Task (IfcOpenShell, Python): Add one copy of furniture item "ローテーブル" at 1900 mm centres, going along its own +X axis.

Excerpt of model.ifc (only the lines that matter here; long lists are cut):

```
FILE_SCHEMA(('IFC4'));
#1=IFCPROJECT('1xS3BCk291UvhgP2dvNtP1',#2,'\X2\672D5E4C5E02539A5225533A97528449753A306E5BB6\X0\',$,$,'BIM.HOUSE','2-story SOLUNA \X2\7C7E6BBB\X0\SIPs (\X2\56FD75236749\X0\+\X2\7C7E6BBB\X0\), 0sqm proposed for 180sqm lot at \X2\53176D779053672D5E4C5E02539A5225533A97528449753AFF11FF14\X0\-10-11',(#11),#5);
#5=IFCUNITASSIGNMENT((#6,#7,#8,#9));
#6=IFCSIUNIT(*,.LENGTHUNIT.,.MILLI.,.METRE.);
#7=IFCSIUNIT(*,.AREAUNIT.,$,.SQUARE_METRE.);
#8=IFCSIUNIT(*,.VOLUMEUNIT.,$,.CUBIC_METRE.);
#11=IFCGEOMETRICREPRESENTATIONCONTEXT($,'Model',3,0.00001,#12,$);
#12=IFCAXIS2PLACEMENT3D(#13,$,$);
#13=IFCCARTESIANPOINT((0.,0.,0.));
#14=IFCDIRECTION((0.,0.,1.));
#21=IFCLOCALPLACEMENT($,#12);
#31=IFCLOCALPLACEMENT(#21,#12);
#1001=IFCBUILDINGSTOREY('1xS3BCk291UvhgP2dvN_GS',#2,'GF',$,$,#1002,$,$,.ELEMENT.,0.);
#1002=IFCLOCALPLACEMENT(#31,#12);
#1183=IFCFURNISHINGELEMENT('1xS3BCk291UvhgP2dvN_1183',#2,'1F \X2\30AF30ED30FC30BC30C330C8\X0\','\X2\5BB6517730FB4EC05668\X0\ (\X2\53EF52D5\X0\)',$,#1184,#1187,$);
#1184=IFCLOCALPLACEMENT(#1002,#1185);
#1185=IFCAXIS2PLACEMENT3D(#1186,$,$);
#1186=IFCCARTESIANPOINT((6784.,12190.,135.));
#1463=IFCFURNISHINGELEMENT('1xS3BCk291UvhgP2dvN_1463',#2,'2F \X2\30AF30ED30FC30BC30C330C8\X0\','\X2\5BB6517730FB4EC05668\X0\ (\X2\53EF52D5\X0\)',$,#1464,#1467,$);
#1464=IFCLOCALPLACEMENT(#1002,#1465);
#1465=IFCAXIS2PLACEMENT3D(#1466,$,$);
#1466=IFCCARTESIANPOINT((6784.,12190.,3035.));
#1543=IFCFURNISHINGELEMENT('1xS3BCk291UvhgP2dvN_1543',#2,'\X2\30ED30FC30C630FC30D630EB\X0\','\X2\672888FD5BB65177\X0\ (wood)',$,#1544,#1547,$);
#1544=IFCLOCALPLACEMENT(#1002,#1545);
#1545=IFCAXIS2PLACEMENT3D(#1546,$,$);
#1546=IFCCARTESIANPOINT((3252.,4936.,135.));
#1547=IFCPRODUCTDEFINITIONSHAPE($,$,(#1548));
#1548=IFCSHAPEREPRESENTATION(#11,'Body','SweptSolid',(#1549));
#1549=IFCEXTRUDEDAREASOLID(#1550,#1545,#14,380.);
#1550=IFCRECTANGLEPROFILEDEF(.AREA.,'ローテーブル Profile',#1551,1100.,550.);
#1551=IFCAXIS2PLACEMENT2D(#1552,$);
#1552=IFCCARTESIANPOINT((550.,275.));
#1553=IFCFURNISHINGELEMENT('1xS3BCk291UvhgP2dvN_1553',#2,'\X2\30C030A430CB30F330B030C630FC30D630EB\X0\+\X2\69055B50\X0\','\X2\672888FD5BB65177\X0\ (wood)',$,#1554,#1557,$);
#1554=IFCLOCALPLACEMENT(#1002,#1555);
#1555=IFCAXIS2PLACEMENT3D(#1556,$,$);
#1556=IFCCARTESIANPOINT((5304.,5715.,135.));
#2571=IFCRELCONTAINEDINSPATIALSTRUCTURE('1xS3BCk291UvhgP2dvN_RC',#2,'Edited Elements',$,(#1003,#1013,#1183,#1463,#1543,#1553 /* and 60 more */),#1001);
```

```python
import ifcopenshell
import ifcopenshell.api.geometry
import ifcopenshell.api.root
import ifcopenshell.util.element
import ifcopenshell.util.placement
import ifcopenshell.util.unit

model = ifcopenshell.open("model.ifc")
unit_scale = ifcopenshell.util.unit.calculate_unit_scale(model)


def reuse_history(source, copy):
    """copy_class also copies each property set's owner history, people and application; keep the originals."""
    for rel in copy.IsDefinedBy:
        if rel.is_a("IfcRelDefinesByProperties") and (history := rel.RelatingPropertyDefinition.OwnerHistory):
            rel.RelatingPropertyDefinition.OwnerHistory = source.OwnerHistory
            ifcopenshell.util.element.remove_deep2(model, history)


source = model.by_id(1543)
base = ifcopenshell.util.placement.get_local_placement(source.ObjectPlacement)
step = base[:3, 0] * 1.9 / unit_scale

for i in range(1, 2):
    copy = ifcopenshell.api.root.copy_class(model, product=source)
    copy.Representation = ifcopenshell.util.element.copy_deep(
        model, source.Representation, exclude=["IfcGeometricRepresentationContext", "IfcRepresentationMap"]
    )
    reuse_history(source, copy)
    matrix = base.copy()
    matrix[:3, 3] += i * step
    print("added at", matrix[:3, 3].round(3) + 0.0)
    ifcopenshell.api.geometry.edit_object_placement(model, product=copy, matrix=matrix, is_si=False)

model.write("model_edited.ifc")
```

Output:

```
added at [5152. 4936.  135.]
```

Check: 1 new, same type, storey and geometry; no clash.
